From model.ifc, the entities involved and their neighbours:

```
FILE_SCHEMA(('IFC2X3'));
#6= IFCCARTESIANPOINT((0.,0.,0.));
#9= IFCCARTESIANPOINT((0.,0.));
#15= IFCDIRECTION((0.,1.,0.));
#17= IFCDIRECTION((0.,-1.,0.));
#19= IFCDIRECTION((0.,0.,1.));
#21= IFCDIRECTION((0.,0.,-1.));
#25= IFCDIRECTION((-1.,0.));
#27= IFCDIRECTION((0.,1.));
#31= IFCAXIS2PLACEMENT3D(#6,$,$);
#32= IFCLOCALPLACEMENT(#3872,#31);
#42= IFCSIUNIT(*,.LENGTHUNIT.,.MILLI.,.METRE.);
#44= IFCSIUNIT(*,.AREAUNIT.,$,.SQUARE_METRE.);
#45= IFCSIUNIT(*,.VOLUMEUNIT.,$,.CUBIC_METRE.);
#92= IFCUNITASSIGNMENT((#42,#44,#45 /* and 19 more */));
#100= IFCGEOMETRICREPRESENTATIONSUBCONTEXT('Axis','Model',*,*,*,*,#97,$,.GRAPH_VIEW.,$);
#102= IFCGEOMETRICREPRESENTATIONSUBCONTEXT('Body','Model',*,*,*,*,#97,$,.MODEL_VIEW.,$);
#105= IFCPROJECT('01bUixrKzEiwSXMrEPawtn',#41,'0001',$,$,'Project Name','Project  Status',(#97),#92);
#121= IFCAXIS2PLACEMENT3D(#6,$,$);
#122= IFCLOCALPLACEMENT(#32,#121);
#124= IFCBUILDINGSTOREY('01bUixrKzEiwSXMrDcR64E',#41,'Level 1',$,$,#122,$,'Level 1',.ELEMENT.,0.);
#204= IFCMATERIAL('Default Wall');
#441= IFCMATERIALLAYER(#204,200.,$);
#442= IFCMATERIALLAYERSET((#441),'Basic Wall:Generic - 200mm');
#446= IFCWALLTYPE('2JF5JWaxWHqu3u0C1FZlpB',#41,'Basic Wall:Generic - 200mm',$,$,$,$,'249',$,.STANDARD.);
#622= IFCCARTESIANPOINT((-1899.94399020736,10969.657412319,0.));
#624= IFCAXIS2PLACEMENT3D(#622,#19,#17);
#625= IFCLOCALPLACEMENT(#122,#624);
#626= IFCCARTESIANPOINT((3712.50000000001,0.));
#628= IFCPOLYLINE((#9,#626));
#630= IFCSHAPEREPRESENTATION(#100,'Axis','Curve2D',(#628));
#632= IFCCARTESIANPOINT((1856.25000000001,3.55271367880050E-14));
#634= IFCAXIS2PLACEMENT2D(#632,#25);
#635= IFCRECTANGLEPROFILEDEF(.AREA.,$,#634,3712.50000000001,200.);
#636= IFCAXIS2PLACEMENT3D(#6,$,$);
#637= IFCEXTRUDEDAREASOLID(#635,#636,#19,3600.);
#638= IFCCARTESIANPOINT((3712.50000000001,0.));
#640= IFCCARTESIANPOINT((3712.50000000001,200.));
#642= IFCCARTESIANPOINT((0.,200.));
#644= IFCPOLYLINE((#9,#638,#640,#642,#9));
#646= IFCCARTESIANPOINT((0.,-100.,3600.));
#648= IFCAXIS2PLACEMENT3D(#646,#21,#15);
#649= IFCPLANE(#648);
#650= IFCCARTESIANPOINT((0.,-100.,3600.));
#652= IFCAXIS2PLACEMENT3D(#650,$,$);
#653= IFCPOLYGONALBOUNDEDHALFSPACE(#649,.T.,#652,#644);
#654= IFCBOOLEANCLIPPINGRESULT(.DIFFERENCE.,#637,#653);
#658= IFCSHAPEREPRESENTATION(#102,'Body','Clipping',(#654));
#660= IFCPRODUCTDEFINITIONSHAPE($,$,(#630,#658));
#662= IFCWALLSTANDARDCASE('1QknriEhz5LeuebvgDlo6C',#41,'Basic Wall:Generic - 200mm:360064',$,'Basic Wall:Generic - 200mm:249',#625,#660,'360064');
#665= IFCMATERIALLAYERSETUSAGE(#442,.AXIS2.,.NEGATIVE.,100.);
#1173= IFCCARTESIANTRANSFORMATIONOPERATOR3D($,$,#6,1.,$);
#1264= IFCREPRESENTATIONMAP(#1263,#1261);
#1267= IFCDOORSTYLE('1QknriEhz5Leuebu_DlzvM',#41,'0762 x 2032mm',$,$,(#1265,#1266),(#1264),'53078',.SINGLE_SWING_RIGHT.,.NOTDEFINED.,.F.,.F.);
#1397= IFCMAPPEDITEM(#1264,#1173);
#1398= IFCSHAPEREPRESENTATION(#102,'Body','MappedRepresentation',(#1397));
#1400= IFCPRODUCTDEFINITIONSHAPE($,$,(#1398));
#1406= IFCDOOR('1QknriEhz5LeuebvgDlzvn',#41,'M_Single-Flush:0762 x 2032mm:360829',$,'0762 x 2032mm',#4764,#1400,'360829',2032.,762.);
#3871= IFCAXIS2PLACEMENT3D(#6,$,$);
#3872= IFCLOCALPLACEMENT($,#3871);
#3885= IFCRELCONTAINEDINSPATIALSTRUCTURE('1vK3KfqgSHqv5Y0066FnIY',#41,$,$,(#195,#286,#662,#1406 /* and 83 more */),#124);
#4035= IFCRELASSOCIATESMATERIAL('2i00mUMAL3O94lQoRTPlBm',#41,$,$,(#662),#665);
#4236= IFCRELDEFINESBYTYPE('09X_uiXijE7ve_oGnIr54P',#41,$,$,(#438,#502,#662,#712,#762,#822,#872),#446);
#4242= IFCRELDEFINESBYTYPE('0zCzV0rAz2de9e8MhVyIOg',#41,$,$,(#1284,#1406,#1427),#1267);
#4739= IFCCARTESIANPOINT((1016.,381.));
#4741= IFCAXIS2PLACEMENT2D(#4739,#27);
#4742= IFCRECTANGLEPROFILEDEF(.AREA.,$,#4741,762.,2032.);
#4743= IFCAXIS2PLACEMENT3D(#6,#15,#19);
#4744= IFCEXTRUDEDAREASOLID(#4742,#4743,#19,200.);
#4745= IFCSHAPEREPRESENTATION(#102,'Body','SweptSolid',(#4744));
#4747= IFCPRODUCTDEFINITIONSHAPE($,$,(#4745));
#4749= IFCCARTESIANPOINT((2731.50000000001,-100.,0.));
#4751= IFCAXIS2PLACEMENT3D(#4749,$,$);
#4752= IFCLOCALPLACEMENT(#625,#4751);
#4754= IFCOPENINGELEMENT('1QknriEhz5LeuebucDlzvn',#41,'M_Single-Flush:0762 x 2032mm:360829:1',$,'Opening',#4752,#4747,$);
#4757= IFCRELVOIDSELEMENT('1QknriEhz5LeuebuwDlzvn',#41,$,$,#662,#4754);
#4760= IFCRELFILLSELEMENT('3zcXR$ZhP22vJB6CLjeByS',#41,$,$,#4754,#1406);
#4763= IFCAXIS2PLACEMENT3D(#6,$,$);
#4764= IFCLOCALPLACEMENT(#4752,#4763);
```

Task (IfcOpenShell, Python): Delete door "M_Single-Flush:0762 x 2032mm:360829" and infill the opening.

```python
import ifcopenshell
import ifcopenshell.api.feature
import ifcopenshell.api.root
import ifcopenshell.geom
import ifcopenshell.util.shape

model = ifcopenshell.open("model.ifc")
settings = ifcopenshell.geom.settings()


def volume(element):
    """Net volume in cubic metres, openings subtracted."""
    shape = ifcopenshell.geom.create_shape(settings, element)
    return ifcopenshell.util.shape.get_volume(shape.geometry)


door = model.by_guid("1QknriEhz5LeuebvgDlzvn")
opening = door.FillsVoids[0].RelatingOpeningElement
wall = opening.VoidsElements[0].RelatingBuildingElement
before = volume(wall)

ifcopenshell.api.root.remove_product(model, product=door)
ifcopenshell.api.feature.remove_feature(model, feature=opening)

after = volume(wall)

print(f"wall volume {before:.3f} -> {after:.3f} m3")

model.write("model_updated.ifc")
```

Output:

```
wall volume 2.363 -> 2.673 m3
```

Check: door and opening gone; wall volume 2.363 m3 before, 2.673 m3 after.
